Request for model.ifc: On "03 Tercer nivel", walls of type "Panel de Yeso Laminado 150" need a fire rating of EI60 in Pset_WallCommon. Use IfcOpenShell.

First a look at what the model holds.

```python
import ifcopenshell
import ifcopenshell.util.element

model = ifcopenshell.open("model.ifc")
print(model.schema)
storey = next(s for s in model.by_type("IfcBuildingStorey") if s.Name == "03 Tercer nivel")
walls = [e for e in ifcopenshell.util.element.get_decomposition(storey) if e.is_a("IfcWall")]
seen = {}
for e in walls:
    element_type = ifcopenshell.util.element.get_type(e)
    key = (element_type.Name if element_type != e and element_type else None, ifcopenshell.util.element.get_pset(e, "Pset_WallCommon", "FireRating"))
    seen[key] = seen.get(key, 0) + 1
for (name, value), count in sorted(seen.items(), key=str):
    print(count, "x", name, "|", value)
```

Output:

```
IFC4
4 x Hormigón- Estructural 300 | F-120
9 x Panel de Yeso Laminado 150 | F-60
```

```python
import ifcopenshell
import ifcopenshell.api.pset
import ifcopenshell.util.element

model = ifcopenshell.open("model.ifc")

storey = next(s for s in model.by_type("IfcBuildingStorey") if s.Name == "03 Tercer nivel")
walls = [e for e in ifcopenshell.util.element.get_decomposition(storey) if e.is_a("IfcWall")]

count = 0
for e in walls:
    element_type = ifcopenshell.util.element.get_type(e)
    if element_type in (None, e) or element_type.Name != "Panel de Yeso Laminado 150":
        continue
    # add_pset returns the element's existing set when there is one.
    pset = ifcopenshell.api.pset.add_pset(model, product=e, name="Pset_WallCommon")
    ifcopenshell.api.pset.edit_pset(model, pset=pset, properties={"FireRating": "EI60"})
    count += 1

print(count, "walls updated")

model.write("model_rev.ifc")
```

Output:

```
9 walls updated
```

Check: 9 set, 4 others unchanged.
